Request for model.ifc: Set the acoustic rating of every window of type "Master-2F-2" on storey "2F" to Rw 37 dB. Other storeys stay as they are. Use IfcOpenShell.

First a look at what the model holds.

```python
import ifcopenshell
import ifcopenshell.util.element

model = ifcopenshell.open("model.ifc")
print(model.schema)
storey = next(s for s in model.by_type("IfcBuildingStorey") if s.Name == "2F")
windows = [e for e in ifcopenshell.util.element.get_decomposition(storey) if e.is_a("IfcWindow")]
seen = {}
for e in windows:
    element_type = ifcopenshell.util.element.get_type(e)
    key = (element_type.Name if element_type != e and element_type else None, ifcopenshell.util.element.get_pset(e, "Pset_WindowCommon", "AcousticRating"))
    seen[key] = seen.get(key, 0) + 1
for (name, value), count in sorted(seen.items(), key=str):
    print(count, "x", name, "|", value)
```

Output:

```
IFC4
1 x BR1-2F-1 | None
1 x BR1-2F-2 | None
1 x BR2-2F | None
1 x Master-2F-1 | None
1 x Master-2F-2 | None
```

```python
import ifcopenshell
import ifcopenshell.api.pset
import ifcopenshell.util.element

model = ifcopenshell.open("model.ifc")

storey = next(s for s in model.by_type("IfcBuildingStorey") if s.Name == "2F")
windows = [e for e in ifcopenshell.util.element.get_decomposition(storey) if e.is_a("IfcWindow")]

count = 0
for e in windows:
    element_type = ifcopenshell.util.element.get_type(e)
    if element_type in (None, e) or element_type.Name != "Master-2F-2":
        continue
    # add_pset returns the element's existing set when there is one.
    pset = ifcopenshell.api.pset.add_pset(model, product=e, name="Pset_WindowCommon")
    ifcopenshell.api.pset.edit_pset(model, pset=pset, properties={"AcousticRating": "Rw 37 dB"})
    count += 1

print(count, "windows updated")

model.write("model_rev.ifc")
```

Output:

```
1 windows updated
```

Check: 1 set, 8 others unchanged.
